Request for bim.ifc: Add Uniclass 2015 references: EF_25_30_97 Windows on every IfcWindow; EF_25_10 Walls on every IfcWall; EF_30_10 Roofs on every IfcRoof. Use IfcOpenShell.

First a look at what the model holds.

```python
import ifcopenshell

model = ifcopenshell.open("bim.ifc")
print(model.schema)
print("classifications:", [c.Name for c in model.by_type("IfcClassification")])
for ifc_class in ("IfcDoor", "IfcRoof", "IfcStair", "IfcWall", "IfcWindow"):
    print(ifc_class, len(model.by_type(ifc_class)))
```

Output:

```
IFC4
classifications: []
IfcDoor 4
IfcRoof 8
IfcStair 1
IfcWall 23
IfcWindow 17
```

```python
import ifcopenshell
import ifcopenshell.api.classification

model = ifcopenshell.open("bim.ifc")

system = ifcopenshell.api.classification.add_classification(model, classification="Uniclass 2015")

codes = {
    "IfcWindow": ("EF_25_30_97", "Windows"),
    "IfcWall": ("EF_25_10", "Walls"),
    "IfcRoof": ("EF_30_10", "Roofs"),
}
for ifc_class, (code, name) in codes.items():
    products = model.by_type(ifc_class)
    ifcopenshell.api.classification.add_reference(
        model, products=products, classification=system, identification=code, name=name
    )
    print(code, len(products))

model.write("bim_rev.ifc")
```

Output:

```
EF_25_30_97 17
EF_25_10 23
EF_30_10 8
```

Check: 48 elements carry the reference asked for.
